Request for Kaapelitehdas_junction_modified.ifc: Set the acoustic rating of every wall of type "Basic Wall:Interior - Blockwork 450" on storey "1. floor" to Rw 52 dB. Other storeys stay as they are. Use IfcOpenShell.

First a look at what the model holds.

```python
import ifcopenshell
import ifcopenshell.util.element

model = ifcopenshell.open("Kaapelitehdas_junction_modified.ifc")
print(model.schema)
storey = next(s for s in model.by_type("IfcBuildingStorey") if s.Name == "1. floor")
walls = [e for e in ifcopenshell.util.element.get_decomposition(storey) if e.is_a("IfcWall")]
seen = {}
for e in walls:
    element_type = ifcopenshell.util.element.get_type(e)
    key = (element_type.Name if element_type != e and element_type else None, ifcopenshell.util.element.get_pset(e, "Pset_WallCommon", "AcousticRating"))
    seen[key] = seen.get(key, 0) + 1
for (name, value), count in sorted(seen.items(), key=str):
    print(count, "x", name, "|", value)
```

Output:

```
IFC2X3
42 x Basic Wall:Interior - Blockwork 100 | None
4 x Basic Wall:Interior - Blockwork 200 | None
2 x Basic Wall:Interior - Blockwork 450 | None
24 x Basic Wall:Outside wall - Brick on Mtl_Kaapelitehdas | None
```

```python
import ifcopenshell
import ifcopenshell.api.pset
import ifcopenshell.util.element

model = ifcopenshell.open("Kaapelitehdas_junction_modified.ifc")

storey = next(s for s in model.by_type("IfcBuildingStorey") if s.Name == "1. floor")
walls = [e for e in ifcopenshell.util.element.get_decomposition(storey) if e.is_a("IfcWall")]

count = 0
for e in walls:
    element_type = ifcopenshell.util.element.get_type(e)
    if element_type in (None, e) or element_type.Name != "Basic Wall:Interior - Blockwork 450":
        continue
    # add_pset returns the element's existing set when there is one.
    pset = ifcopenshell.api.pset.add_pset(model, product=e, name="Pset_WallCommon")
    ifcopenshell.api.pset.edit_pset(model, pset=pset, properties={"AcousticRating": "Rw 52 dB"})
    count += 1

print(count, "walls updated")

model.write("Kaapelitehdas_junction_modified_rev.ifc")
```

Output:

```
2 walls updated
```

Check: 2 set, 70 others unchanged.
